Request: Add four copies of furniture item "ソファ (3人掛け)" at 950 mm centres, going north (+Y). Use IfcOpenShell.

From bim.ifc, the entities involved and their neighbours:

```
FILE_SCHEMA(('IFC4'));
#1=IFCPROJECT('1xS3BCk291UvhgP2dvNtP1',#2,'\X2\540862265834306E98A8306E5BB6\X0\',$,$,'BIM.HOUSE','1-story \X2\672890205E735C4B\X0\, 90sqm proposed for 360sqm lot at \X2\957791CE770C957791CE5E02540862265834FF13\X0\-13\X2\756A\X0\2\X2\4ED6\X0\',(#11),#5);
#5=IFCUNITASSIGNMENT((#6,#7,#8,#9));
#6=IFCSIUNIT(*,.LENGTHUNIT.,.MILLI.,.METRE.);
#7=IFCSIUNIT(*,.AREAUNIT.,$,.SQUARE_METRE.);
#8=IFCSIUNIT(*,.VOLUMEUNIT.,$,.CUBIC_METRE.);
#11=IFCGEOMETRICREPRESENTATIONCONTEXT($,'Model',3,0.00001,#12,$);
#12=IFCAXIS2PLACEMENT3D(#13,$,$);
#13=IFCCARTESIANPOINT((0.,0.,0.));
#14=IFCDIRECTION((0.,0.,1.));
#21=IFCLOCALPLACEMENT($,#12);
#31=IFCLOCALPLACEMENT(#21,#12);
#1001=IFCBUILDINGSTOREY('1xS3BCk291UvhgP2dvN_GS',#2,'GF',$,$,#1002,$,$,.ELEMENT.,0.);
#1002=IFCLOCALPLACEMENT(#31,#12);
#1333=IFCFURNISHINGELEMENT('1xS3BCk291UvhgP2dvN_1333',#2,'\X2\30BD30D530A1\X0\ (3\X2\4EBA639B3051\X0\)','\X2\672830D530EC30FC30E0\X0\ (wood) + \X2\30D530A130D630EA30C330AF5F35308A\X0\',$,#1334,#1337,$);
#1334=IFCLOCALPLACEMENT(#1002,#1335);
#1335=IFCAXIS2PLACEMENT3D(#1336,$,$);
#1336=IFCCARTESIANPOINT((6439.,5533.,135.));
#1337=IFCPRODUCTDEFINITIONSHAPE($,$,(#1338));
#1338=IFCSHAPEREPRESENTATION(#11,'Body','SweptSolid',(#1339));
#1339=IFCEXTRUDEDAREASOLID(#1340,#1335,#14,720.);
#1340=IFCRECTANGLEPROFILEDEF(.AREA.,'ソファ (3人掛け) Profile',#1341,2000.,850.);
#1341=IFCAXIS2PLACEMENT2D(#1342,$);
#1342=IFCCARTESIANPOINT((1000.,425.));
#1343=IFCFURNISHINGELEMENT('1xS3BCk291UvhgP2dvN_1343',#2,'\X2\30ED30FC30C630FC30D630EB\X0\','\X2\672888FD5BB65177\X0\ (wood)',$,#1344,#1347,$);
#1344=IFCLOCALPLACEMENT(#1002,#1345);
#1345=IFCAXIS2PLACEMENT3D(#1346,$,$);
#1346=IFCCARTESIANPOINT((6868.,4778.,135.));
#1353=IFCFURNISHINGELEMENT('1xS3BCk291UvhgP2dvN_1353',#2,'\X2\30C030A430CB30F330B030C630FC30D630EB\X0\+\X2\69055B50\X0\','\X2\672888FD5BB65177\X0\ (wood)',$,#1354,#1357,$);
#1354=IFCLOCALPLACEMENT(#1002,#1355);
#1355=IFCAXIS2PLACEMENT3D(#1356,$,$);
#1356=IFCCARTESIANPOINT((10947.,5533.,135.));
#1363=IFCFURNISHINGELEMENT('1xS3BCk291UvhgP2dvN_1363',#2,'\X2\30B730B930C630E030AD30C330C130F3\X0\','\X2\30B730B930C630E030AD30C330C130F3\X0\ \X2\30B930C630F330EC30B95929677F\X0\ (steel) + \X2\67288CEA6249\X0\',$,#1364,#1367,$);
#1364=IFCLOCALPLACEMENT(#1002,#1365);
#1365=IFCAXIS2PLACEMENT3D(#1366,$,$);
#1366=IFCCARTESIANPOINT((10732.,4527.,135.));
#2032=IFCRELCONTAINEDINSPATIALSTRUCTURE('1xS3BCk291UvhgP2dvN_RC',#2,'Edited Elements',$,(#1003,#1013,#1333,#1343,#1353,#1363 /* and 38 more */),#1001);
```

```python
import numpy as np
import ifcopenshell
import ifcopenshell.api.geometry
import ifcopenshell.api.root
import ifcopenshell.util.element
import ifcopenshell.util.placement

model = ifcopenshell.open("bim.ifc")


def reuse_history(source, copy):
    """copy_class also copies each property set's owner history, people and application; keep the originals."""
    for rel in copy.IsDefinedBy:
        if rel.is_a("IfcRelDefinesByProperties") and (history := rel.RelatingPropertyDefinition.OwnerHistory):
            rel.RelatingPropertyDefinition.OwnerHistory = source.OwnerHistory
            ifcopenshell.util.element.remove_deep2(model, history)


source = model.by_guid("1xS3BCk291UvhgP2dvN_1333")
base = ifcopenshell.util.placement.get_local_placement(source.ObjectPlacement)
step = np.array([0.0, 1.0, 0.0]) * 950.0

for i in range(1, 5):
    copy = ifcopenshell.api.root.copy_class(model, product=source)
    copy.Representation = ifcopenshell.util.element.copy_deep(
        model, source.Representation, exclude=["IfcGeometricRepresentationContext", "IfcRepresentationMap"]
    )
    reuse_history(source, copy)
    matrix = base.copy()
    matrix[:3, 3] += i * step
    print("added at", matrix[:3, 3].round(3) + 0.0)
    ifcopenshell.api.geometry.edit_object_placement(model, product=copy, matrix=matrix, is_si=False)

model.write("bim-out.ifc")
```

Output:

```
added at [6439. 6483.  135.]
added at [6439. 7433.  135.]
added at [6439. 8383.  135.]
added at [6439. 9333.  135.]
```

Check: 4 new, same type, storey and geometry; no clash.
